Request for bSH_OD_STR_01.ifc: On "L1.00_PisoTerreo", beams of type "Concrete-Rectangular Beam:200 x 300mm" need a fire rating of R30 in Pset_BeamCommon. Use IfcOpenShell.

First a look at what the model holds.

```python
import ifcopenshell
import ifcopenshell.util.element

model = ifcopenshell.open("bSH_OD_STR_01.ifc")
print(model.schema)
storey = next(s for s in model.by_type("IfcBuildingStorey") if s.Name == "L1.00_PisoTerreo")
beams = [e for e in ifcopenshell.util.element.get_decomposition(storey) if e.is_a("IfcBeam")]
seen = {}
for e in beams:
    element_type = ifcopenshell.util.element.get_type(e)
    key = (element_type.Name if element_type != e and element_type else None, ifcopenshell.util.element.get_pset(e, "Pset_BeamCommon", "FireRating"))
    seen[key] = seen.get(key, 0) + 1
for (name, value), count in sorted(seen.items(), key=str):
    print(count, "x", name, "|", value)
```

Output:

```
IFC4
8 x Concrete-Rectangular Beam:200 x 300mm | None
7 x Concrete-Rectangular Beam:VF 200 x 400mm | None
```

```python
import ifcopenshell
import ifcopenshell.api.pset
import ifcopenshell.util.element

model = ifcopenshell.open("bSH_OD_STR_01.ifc")

storey = next(s for s in model.by_type("IfcBuildingStorey") if s.Name == "L1.00_PisoTerreo")
beams = [e for e in ifcopenshell.util.element.get_decomposition(storey) if e.is_a("IfcBeam")]

count = 0
for e in beams:
    element_type = ifcopenshell.util.element.get_type(e)
    if element_type in (None, e) or element_type.Name != "Concrete-Rectangular Beam:200 x 300mm":
        continue
    # add_pset returns the element's existing set when there is one.
    pset = ifcopenshell.api.pset.add_pset(model, product=e, name="Pset_BeamCommon")
    ifcopenshell.api.pset.edit_pset(model, pset=pset, properties={"FireRating": "R30"})
    count += 1

print(count, "beams updated")

model.write("bSH_OD_STR_01_edited.ifc")
```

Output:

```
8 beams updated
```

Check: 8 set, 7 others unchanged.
